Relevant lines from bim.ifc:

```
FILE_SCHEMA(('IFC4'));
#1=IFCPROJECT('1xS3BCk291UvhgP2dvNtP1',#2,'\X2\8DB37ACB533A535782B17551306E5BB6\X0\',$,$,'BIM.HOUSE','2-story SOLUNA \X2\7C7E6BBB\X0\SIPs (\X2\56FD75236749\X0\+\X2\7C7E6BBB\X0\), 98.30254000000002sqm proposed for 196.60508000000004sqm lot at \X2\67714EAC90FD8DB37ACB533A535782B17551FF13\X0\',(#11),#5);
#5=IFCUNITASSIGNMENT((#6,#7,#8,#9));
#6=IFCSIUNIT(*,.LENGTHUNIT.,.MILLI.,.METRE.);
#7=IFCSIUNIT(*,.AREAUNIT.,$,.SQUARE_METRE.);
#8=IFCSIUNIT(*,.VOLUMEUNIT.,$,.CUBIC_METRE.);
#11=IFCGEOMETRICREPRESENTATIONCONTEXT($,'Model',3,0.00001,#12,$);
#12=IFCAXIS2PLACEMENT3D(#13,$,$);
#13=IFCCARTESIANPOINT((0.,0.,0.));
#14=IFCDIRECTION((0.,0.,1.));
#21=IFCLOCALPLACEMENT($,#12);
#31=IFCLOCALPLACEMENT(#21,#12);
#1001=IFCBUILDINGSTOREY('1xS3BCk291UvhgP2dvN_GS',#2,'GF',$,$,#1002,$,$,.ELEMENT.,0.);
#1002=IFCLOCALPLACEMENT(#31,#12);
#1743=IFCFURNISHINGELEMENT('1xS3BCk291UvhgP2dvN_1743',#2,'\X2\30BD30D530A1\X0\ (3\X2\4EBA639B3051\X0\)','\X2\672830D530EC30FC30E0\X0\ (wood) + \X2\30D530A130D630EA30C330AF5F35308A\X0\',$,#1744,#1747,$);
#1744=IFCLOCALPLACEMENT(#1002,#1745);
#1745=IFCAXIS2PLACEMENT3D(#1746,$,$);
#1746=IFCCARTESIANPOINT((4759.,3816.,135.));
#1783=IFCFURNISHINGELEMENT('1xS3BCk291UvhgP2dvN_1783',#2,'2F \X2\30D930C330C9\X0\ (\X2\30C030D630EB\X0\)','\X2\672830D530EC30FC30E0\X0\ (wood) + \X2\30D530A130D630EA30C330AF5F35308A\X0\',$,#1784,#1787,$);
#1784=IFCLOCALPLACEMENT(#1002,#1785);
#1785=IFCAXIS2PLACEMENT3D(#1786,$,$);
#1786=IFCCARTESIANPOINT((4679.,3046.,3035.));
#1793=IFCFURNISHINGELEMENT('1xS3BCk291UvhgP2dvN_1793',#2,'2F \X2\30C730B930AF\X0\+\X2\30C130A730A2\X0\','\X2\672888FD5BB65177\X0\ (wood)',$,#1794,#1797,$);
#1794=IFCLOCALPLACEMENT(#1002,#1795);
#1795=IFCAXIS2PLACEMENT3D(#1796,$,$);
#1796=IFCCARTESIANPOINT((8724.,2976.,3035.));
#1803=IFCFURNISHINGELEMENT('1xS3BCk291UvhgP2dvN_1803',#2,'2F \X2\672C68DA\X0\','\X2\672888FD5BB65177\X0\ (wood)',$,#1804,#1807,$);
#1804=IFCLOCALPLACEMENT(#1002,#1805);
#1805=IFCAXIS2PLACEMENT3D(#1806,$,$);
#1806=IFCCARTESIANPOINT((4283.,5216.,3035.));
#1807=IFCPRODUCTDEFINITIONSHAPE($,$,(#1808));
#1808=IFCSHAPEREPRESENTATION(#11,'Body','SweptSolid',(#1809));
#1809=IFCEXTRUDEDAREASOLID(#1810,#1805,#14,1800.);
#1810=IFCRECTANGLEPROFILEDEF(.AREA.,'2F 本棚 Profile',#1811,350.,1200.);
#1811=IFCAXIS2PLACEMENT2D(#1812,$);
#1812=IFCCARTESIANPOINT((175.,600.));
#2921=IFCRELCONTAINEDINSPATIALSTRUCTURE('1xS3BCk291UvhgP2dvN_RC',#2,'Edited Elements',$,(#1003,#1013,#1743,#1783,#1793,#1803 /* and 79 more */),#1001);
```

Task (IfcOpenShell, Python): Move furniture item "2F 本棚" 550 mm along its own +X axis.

```python
import ifcopenshell
import ifcopenshell.api.geometry
import ifcopenshell.util.placement

model = ifcopenshell.open("bim.ifc")

item = model.by_guid("1xS3BCk291UvhgP2dvN_1803")
matrix = ifcopenshell.util.placement.get_local_placement(item.ObjectPlacement)
matrix[:3, 3] += matrix[:3, 0] * 550.0
ifcopenshell.api.geometry.edit_object_placement(model, product=item, matrix=matrix, is_si=False)

print(ifcopenshell.util.placement.get_local_placement(item.ObjectPlacement).round(3) + 0.0)

model.write("bim-out.ifc")
```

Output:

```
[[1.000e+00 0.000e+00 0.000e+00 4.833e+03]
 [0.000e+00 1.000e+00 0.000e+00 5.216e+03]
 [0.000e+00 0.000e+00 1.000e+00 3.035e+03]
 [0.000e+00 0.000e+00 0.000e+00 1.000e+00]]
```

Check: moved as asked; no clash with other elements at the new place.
